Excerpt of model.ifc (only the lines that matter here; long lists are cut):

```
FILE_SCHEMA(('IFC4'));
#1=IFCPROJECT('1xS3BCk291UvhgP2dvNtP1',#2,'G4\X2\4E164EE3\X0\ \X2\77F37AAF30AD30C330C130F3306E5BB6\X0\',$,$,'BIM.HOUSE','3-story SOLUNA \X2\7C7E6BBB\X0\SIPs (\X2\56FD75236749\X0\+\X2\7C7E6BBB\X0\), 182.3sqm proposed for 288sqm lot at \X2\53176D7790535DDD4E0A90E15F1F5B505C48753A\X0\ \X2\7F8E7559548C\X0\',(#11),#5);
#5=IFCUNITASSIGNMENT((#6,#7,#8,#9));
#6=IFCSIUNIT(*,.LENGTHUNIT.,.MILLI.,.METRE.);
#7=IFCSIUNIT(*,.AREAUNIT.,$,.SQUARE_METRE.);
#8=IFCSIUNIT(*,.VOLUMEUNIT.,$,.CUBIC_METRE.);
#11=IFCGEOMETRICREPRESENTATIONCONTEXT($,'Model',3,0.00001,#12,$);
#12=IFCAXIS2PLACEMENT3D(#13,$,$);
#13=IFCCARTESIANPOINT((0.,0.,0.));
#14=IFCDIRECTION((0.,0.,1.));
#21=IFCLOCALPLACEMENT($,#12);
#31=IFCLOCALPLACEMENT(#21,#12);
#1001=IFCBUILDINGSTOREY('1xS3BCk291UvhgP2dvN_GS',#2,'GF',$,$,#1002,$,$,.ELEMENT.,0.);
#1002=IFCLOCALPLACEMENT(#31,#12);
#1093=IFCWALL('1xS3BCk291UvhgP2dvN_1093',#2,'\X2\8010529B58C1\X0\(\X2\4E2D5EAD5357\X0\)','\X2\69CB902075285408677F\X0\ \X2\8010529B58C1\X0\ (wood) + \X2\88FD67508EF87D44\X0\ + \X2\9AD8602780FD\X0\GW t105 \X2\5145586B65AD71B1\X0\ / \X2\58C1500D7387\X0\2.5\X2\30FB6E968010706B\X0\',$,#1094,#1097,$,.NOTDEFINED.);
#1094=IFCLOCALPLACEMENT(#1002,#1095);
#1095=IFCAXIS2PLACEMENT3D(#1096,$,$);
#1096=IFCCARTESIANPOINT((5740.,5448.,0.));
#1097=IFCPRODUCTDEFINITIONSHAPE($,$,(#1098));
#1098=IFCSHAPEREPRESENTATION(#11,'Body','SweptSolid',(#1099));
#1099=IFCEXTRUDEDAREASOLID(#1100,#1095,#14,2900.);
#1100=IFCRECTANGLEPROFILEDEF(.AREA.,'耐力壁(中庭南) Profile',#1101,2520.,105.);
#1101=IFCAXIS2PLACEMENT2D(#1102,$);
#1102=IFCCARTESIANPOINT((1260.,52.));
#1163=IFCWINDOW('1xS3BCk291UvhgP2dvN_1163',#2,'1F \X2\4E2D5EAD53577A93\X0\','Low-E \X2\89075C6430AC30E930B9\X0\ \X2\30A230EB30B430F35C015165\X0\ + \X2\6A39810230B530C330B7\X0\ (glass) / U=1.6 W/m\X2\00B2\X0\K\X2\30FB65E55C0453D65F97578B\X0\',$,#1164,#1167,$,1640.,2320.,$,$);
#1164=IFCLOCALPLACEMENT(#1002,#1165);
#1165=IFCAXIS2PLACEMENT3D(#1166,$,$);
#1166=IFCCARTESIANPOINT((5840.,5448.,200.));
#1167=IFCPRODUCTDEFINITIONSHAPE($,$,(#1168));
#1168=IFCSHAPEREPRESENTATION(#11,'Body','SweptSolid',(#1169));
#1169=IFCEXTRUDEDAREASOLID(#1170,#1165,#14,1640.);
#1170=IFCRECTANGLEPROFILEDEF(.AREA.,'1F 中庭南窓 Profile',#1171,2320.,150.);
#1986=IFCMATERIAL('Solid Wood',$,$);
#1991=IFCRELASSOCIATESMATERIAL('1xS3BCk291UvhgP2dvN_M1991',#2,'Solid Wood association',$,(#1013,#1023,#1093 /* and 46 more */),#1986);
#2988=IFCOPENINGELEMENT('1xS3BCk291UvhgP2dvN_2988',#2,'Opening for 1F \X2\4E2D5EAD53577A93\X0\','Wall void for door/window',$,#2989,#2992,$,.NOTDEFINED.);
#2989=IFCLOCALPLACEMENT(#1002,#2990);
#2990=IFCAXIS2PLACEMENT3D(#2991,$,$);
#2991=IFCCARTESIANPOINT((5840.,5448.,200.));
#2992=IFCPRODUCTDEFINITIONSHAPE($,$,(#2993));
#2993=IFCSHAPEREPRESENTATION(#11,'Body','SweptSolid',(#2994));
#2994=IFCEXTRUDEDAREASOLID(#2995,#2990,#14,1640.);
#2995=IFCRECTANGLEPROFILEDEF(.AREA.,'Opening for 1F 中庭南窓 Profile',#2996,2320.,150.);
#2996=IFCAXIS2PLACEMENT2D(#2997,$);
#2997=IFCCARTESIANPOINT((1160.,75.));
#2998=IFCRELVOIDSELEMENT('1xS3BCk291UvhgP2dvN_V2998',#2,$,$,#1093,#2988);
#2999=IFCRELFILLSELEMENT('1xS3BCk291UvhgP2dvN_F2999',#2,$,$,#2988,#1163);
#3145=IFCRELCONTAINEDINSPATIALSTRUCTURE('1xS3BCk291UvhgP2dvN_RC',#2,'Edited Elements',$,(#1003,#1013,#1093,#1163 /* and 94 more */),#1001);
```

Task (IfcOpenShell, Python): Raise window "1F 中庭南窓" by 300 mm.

```python
import numpy as np
import ifcopenshell
import ifcopenshell.api.geometry
import ifcopenshell.util.placement
import ifcopenshell.util.unit

model = ifcopenshell.open("model.ifc")
unit_scale = ifcopenshell.util.unit.calculate_unit_scale(model)

window = model.by_id(1163)
opening = window.FillsVoids[0].RelatingOpeningElement
dz = 0.3 / unit_scale

shift = np.array([0.0, 0.0, dz])
# The window is not placed relative to its opening, so move both.
for product in (opening, window):
    matrix = ifcopenshell.util.placement.get_local_placement(product.ObjectPlacement)
    matrix[:3, 3] += shift
    ifcopenshell.api.geometry.edit_object_placement(model, product=product, matrix=matrix, is_si=False)

print(f"moved by {dz * unit_scale:+.3f} m")

model.write("model_edited.ifc")
```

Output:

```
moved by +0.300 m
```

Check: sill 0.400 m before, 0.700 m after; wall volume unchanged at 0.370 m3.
